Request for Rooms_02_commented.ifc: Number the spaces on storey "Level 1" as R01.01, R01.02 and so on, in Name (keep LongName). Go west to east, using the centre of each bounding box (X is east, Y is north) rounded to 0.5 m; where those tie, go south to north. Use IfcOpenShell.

First a look at what the model holds.

```python
import ifcopenshell
import ifcopenshell.util.element
import ifcopenshell.util.placement

model = ifcopenshell.open("Rooms_02_commented.ifc")
print(model.schema)
storey = next(s for s in model.by_type("IfcBuildingStorey") if s.Name == "Level 1")
spaces = [e for e in ifcopenshell.util.element.get_decomposition(storey) if e.is_a("IfcSpace")]
for e in sorted(spaces, key=lambda e: e.id()):
    origin = ifcopenshell.util.placement.get_local_placement(e.ObjectPlacement)[:3, 3]
    print(e.id(), e.Name, e.LongName, origin.round(2) + 0.0, sep=" | ")
```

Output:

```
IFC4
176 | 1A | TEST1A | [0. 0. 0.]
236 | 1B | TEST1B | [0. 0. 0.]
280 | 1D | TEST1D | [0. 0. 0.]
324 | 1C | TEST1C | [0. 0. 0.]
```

```python
import ifcopenshell
import ifcopenshell.geom
import ifcopenshell.util.element
import ifcopenshell.util.shape

model = ifcopenshell.open("Rooms_02_commented.ifc")
settings = ifcopenshell.geom.settings()
settings.set("use-world-coords", True)


def centre(element):
    shape = ifcopenshell.geom.create_shape(settings, element)
    return ifcopenshell.util.shape.get_bbox_centroid(shape.geometry)


storey = next(s for s in model.by_type("IfcBuildingStorey") if s.Name == "Level 1")
spaces = [e for e in ifcopenshell.util.element.get_decomposition(storey) if e.is_a("IfcSpace")]

# Insertion points can sit at a corner or the storey origin, so sort by the geometry (in metres).
centres = {e: centre(e) for e in spaces}
spaces.sort(key=lambda e: (round(centres[e][0] / 0.5), centres[e][1]))

for i, e in enumerate(spaces, start=1):
    number = f"R01.{i:02d}"
    e.Name = number
    print(e.id(), number)

model.write("Rooms_02_commented_updated.ifc")
```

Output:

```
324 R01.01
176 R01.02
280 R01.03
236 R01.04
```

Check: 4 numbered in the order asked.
